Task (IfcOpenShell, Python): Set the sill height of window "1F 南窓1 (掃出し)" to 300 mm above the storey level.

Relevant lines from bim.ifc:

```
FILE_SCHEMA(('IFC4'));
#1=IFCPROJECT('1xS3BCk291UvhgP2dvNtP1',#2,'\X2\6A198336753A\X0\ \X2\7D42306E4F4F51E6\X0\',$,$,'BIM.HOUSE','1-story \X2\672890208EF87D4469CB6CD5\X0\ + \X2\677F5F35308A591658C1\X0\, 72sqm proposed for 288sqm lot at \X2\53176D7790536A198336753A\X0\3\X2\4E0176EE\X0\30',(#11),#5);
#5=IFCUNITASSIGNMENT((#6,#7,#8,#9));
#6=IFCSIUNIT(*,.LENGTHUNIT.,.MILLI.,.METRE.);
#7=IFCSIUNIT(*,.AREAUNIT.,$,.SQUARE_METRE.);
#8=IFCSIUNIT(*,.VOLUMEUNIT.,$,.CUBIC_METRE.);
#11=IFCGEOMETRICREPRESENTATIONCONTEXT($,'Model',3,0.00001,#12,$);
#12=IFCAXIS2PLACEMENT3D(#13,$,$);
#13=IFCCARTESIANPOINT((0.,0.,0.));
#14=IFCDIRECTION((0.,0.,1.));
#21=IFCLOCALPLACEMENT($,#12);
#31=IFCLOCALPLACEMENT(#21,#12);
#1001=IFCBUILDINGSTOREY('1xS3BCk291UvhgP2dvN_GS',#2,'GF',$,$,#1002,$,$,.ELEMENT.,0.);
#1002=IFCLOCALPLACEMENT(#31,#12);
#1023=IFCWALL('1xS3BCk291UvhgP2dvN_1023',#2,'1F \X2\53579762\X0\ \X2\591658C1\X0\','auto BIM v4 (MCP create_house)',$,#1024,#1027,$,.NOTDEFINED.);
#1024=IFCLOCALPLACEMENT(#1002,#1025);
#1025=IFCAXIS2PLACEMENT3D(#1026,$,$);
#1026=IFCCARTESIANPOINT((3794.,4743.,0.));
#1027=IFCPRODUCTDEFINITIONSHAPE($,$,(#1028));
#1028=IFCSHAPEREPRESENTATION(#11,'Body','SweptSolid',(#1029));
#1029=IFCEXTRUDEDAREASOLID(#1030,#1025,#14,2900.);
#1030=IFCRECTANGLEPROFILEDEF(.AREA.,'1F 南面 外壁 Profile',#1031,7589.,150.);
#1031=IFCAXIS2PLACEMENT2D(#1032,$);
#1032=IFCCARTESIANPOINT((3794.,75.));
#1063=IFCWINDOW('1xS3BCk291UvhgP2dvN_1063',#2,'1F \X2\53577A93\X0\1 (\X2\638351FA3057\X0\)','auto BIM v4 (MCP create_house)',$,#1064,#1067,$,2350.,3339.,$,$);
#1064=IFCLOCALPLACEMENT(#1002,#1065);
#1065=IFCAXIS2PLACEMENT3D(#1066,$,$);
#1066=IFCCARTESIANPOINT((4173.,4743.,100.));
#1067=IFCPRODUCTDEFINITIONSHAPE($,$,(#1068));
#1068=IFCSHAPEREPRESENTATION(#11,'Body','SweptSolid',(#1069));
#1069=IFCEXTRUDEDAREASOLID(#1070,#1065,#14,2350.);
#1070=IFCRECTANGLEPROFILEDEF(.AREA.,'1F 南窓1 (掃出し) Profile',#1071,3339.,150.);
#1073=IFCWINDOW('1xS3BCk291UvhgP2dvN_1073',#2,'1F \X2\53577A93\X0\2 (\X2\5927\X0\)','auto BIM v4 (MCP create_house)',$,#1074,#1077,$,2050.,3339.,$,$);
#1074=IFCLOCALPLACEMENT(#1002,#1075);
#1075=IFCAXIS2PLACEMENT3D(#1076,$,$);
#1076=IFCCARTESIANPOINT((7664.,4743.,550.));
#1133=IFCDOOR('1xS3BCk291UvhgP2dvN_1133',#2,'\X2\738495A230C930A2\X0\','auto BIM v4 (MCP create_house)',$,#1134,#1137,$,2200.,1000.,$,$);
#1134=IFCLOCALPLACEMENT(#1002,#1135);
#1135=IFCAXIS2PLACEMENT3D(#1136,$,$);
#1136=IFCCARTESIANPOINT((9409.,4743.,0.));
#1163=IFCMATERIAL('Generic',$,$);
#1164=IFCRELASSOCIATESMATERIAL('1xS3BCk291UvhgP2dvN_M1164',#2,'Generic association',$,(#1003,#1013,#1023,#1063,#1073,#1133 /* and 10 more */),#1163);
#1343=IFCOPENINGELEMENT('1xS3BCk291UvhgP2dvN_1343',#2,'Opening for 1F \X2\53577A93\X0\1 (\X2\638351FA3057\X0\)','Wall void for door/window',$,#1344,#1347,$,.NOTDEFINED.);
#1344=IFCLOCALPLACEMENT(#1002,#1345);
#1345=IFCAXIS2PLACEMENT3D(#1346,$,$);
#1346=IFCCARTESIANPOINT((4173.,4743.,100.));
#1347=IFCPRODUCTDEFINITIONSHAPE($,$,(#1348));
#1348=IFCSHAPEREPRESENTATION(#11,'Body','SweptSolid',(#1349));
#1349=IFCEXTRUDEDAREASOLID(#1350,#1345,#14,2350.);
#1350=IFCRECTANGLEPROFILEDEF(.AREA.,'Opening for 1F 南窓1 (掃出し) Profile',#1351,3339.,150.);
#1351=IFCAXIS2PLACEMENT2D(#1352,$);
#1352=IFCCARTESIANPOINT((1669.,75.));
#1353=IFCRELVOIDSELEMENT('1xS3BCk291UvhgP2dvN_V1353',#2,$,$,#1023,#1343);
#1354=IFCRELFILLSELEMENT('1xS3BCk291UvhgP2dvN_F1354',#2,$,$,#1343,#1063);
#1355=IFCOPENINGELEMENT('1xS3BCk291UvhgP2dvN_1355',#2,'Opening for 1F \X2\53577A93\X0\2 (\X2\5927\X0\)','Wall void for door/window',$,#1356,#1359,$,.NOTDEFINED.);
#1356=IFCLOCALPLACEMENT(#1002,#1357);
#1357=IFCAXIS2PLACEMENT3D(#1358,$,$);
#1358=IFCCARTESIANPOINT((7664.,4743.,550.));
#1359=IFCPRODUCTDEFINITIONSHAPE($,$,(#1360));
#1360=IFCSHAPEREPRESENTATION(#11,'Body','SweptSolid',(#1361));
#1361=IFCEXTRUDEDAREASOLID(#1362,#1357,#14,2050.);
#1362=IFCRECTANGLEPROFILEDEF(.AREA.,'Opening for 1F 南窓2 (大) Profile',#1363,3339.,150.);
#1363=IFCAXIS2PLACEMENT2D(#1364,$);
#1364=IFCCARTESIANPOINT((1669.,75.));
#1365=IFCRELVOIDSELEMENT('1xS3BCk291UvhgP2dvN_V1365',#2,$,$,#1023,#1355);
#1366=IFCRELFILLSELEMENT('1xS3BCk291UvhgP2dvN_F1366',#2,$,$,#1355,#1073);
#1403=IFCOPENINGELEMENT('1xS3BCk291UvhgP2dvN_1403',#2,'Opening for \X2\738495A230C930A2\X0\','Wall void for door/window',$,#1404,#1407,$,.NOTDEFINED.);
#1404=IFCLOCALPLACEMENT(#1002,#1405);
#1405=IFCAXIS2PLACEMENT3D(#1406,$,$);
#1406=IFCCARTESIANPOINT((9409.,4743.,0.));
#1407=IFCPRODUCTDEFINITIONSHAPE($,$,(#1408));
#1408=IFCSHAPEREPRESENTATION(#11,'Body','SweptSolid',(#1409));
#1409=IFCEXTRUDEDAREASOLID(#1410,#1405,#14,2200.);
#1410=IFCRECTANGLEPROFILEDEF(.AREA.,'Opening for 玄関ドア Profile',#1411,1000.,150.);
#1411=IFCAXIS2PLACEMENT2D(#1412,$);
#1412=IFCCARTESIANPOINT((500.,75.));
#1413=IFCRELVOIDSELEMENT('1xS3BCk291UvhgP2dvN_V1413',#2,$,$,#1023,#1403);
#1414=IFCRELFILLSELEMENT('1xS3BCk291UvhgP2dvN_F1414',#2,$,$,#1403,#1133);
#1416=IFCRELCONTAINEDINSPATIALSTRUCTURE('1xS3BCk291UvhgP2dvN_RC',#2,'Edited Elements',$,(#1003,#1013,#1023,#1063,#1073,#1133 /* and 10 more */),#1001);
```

```python
import numpy as np
import ifcopenshell
import ifcopenshell.api.geometry
import ifcopenshell.geom
import ifcopenshell.util.element
import ifcopenshell.util.placement
import ifcopenshell.util.shape
import ifcopenshell.util.unit

model = ifcopenshell.open("bim.ifc")
unit_scale = ifcopenshell.util.unit.calculate_unit_scale(model)

window = model.by_id(1063)
opening = window.FillsVoids[0].RelatingOpeningElement
storey = ifcopenshell.util.element.get_container(window, ifc_class="IfcBuildingStorey")
level = ifcopenshell.util.placement.get_local_placement(storey.ObjectPlacement)[2, 3]

# The opening's origin need not be at the sill, so measure its lowest point.
shape = ifcopenshell.geom.create_shape(ifcopenshell.geom.settings(), opening)
bottom = ifcopenshell.util.shape.get_shape_bottom_elevation(shape, shape.geometry) / unit_scale
dz = level + 0.3 / unit_scale - bottom

shift = np.array([0.0, 0.0, dz])
# The window is not placed relative to its opening, so move both.
for product in (opening, window):
    matrix = ifcopenshell.util.placement.get_local_placement(product.ObjectPlacement)
    matrix[:3, 3] += shift
    ifcopenshell.api.geometry.edit_object_placement(model, product=product, matrix=matrix, is_si=False)

print(f"moved by {dz * unit_scale:+.3f} m")

model.write("bim_v2.ifc")
```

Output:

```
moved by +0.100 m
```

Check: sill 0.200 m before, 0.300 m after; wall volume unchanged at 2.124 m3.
